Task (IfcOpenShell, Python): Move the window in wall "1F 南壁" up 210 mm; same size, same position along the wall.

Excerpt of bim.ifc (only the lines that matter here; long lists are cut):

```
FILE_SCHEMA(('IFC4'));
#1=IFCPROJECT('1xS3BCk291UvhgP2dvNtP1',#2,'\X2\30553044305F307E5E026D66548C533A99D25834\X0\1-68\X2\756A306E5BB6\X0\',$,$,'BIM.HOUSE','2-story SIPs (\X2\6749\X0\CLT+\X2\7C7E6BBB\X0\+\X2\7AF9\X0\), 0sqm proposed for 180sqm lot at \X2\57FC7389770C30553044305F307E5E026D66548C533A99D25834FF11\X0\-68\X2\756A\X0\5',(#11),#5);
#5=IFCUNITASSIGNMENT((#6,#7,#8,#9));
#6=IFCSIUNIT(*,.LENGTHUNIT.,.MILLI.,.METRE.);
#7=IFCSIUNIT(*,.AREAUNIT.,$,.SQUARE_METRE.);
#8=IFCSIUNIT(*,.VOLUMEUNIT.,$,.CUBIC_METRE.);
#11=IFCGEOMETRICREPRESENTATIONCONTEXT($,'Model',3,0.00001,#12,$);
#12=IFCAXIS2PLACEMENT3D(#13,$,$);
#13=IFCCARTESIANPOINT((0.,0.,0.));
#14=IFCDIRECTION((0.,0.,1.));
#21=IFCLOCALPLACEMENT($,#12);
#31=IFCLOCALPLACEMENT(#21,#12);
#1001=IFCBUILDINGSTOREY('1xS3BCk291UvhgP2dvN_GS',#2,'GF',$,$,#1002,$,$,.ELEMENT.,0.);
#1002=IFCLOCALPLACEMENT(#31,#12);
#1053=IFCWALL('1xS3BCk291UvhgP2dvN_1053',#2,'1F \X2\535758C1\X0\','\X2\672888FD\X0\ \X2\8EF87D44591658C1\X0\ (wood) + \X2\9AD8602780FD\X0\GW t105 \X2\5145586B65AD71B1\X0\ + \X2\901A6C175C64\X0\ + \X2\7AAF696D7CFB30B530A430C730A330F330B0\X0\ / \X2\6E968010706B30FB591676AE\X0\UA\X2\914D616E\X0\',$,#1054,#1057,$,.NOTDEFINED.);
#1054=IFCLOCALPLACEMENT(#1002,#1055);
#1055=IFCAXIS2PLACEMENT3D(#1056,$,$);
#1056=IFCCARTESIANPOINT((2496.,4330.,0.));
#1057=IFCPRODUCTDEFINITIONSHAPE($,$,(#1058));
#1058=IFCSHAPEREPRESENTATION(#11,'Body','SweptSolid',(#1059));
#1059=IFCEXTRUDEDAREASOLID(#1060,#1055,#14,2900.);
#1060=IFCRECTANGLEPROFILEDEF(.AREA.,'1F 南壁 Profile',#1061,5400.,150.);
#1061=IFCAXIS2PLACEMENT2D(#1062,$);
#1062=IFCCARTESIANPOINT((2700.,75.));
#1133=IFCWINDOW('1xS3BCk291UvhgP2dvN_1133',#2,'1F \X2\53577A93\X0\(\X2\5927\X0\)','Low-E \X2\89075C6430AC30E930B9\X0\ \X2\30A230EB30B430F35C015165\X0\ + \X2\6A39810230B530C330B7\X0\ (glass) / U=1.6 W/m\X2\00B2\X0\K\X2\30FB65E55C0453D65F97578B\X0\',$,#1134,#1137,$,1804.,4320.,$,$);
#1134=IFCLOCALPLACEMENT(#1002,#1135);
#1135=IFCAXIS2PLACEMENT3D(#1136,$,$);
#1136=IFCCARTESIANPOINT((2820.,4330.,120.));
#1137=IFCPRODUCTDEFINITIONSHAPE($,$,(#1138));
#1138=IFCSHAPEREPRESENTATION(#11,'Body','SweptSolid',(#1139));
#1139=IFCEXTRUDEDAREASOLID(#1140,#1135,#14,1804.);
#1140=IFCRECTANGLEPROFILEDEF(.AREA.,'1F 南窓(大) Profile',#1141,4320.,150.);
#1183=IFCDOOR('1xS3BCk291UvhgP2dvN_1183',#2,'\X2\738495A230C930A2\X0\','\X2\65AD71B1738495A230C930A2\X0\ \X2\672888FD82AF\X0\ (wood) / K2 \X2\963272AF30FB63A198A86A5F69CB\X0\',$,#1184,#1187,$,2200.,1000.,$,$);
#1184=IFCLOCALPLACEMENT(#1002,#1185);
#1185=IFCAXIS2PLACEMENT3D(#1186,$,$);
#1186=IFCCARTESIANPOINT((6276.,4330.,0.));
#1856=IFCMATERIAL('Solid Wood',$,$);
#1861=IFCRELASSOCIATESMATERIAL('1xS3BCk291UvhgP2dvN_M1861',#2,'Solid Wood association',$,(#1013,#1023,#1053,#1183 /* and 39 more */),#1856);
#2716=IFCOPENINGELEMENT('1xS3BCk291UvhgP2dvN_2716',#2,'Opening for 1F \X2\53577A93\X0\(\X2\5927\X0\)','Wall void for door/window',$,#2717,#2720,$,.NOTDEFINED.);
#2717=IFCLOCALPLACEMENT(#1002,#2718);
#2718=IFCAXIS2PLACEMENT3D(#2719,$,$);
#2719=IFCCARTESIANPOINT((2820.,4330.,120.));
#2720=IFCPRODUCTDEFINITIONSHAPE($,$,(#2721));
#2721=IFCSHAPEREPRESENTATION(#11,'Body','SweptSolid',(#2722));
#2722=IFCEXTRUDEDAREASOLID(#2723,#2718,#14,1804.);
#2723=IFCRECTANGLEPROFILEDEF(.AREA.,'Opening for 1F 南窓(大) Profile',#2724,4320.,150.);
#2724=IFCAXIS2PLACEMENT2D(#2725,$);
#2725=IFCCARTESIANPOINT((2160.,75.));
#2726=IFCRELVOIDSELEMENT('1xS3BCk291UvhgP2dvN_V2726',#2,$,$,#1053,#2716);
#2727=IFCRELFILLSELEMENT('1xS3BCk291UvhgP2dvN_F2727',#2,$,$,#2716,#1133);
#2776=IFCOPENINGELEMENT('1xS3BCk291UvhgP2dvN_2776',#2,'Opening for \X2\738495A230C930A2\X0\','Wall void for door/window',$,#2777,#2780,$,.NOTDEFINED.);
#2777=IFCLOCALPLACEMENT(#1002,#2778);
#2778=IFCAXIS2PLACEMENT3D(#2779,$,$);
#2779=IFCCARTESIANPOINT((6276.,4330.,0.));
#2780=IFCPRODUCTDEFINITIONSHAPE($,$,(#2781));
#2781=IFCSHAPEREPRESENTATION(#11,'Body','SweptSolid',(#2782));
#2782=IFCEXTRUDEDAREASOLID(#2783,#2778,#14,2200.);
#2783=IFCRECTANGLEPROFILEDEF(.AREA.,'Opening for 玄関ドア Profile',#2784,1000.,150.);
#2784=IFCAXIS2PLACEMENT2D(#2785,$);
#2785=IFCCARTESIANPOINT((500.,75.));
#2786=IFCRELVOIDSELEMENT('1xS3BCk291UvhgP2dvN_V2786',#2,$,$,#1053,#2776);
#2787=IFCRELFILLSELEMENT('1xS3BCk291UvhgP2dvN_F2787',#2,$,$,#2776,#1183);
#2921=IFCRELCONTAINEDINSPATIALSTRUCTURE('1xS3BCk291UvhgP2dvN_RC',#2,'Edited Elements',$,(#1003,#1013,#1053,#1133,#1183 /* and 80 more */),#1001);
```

```python
import numpy as np
import ifcopenshell
import ifcopenshell.api.geometry
import ifcopenshell.util.placement
import ifcopenshell.util.unit

model = ifcopenshell.open("bim.ifc")
unit_scale = ifcopenshell.util.unit.calculate_unit_scale(model)

window = model.by_id(1133)
opening = window.FillsVoids[0].RelatingOpeningElement
dz = 0.21 / unit_scale

shift = np.array([0.0, 0.0, dz])
# The window is not placed relative to its opening, so move both.
for product in (opening, window):
    matrix = ifcopenshell.util.placement.get_local_placement(product.ObjectPlacement)
    matrix[:3, 3] += shift
    ifcopenshell.api.geometry.edit_object_placement(model, product=product, matrix=matrix, is_si=False)

print(f"moved by {dz * unit_scale:+.3f} m")

model.write("bim_edited.ifc")
```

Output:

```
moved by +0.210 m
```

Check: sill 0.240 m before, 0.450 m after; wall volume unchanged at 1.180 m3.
